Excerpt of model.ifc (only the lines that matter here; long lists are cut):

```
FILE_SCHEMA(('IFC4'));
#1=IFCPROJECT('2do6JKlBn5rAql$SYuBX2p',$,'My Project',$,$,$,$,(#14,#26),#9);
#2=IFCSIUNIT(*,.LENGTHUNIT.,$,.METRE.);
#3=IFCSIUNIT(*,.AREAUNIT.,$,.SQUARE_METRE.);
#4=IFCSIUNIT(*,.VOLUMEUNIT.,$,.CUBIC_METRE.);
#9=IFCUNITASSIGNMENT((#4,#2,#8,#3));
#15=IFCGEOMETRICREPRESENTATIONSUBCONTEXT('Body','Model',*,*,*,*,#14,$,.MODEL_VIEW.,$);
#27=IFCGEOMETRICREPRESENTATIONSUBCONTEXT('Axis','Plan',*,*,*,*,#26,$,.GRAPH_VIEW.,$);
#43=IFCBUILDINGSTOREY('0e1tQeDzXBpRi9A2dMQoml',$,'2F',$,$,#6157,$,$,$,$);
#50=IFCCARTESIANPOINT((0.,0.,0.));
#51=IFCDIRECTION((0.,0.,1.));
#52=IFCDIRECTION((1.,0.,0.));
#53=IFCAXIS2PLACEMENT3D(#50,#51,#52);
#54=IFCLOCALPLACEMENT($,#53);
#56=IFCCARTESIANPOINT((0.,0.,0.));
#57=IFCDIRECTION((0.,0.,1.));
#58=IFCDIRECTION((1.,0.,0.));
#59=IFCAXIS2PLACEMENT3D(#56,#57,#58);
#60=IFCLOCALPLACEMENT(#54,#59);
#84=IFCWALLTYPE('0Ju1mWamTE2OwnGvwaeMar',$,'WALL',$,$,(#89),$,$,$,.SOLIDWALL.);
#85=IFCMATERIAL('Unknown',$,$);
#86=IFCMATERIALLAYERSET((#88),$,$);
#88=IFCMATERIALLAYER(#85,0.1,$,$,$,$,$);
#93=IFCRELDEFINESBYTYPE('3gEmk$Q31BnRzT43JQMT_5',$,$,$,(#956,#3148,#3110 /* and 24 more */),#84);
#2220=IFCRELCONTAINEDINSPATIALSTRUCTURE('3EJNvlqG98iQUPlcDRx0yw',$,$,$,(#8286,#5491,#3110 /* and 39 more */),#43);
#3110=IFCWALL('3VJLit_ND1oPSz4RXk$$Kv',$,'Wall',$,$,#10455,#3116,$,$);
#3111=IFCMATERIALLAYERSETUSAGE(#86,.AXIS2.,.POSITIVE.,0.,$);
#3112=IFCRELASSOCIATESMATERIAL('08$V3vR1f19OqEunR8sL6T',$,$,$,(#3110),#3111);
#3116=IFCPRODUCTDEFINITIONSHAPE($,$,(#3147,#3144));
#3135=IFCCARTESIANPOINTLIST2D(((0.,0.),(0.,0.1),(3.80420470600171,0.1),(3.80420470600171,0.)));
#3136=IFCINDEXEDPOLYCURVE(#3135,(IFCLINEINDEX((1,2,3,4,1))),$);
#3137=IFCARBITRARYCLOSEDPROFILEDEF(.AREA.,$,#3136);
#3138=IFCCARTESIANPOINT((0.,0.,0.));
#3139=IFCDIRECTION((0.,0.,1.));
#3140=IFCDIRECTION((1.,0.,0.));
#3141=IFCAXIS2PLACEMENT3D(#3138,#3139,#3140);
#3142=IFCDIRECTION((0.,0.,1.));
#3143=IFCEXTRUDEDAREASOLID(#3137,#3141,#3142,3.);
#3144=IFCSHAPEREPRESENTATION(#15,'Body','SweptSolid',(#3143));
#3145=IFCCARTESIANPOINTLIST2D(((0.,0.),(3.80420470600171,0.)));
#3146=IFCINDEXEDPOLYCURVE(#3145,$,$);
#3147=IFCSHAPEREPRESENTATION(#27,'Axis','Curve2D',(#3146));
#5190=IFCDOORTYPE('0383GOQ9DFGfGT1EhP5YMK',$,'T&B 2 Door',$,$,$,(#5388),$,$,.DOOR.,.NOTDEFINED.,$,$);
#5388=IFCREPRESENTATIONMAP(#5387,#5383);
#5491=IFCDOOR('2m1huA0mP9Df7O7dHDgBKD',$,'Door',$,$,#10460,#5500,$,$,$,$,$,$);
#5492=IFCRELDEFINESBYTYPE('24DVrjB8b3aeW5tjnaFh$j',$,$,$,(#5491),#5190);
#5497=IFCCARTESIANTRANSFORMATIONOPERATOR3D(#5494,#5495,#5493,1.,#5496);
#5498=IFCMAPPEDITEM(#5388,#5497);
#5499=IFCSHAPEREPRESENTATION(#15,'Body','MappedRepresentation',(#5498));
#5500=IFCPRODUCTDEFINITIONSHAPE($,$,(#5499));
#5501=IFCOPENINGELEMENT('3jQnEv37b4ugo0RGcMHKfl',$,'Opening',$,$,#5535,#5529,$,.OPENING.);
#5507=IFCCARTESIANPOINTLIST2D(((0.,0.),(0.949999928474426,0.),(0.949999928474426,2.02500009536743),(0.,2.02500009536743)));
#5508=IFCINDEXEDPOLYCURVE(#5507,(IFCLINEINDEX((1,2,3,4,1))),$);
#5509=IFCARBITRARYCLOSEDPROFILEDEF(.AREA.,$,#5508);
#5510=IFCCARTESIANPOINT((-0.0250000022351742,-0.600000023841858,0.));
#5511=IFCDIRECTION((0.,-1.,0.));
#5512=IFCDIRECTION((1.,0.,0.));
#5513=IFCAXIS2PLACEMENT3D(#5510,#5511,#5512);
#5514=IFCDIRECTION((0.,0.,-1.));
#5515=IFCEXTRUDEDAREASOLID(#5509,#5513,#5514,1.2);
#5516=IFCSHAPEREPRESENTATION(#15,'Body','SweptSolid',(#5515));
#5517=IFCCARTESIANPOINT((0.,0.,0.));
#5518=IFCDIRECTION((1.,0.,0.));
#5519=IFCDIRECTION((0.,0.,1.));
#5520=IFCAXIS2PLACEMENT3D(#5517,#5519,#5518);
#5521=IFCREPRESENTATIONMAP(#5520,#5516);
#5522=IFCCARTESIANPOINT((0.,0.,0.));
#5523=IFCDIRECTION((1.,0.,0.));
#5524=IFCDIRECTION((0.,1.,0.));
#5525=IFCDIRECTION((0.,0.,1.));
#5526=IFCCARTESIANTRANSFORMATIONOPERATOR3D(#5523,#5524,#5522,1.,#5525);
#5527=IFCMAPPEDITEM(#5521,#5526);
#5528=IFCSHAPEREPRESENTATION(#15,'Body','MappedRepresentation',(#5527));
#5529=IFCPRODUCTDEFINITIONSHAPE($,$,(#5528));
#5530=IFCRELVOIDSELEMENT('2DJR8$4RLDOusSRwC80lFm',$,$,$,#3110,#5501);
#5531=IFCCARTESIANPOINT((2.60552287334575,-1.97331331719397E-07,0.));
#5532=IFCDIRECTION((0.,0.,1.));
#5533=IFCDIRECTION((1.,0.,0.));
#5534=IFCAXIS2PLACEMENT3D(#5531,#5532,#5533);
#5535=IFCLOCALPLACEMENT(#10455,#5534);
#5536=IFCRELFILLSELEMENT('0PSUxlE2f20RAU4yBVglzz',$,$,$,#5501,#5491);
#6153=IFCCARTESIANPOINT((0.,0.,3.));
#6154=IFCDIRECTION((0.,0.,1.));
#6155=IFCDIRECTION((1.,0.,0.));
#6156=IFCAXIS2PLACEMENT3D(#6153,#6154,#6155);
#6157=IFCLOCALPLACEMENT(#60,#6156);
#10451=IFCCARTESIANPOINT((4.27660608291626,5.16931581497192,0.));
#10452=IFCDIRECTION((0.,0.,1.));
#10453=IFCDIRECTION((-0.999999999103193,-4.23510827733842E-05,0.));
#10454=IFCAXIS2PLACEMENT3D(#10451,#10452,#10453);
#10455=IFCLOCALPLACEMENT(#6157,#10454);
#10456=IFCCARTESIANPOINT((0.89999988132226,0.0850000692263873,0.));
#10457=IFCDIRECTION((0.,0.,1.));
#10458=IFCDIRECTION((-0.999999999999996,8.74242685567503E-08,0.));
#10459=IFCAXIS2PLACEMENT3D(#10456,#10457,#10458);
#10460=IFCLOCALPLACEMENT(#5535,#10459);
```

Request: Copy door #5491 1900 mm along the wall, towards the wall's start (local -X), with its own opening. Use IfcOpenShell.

```python
import ifcopenshell
import ifcopenshell.api.feature
import ifcopenshell.api.geometry
import ifcopenshell.api.root
import ifcopenshell.geom
import ifcopenshell.util.element
import ifcopenshell.util.placement
import ifcopenshell.util.shape
import ifcopenshell.util.unit

model = ifcopenshell.open("model.ifc")
unit_scale = ifcopenshell.util.unit.calculate_unit_scale(model)
settings = ifcopenshell.geom.settings()


def volume(element):
    """Net volume in cubic metres, openings subtracted."""
    shape = ifcopenshell.geom.create_shape(settings, element)
    return ifcopenshell.util.shape.get_volume(shape.geometry)


door = model.by_guid("2m1huA0mP9Df7O7dHDgBKD")
opening = door.FillsVoids[0].RelatingOpeningElement
wall = opening.VoidsElements[0].RelatingBuildingElement
before = volume(wall)
shift = ifcopenshell.util.placement.get_local_placement(wall.ObjectPlacement)[:3, 0] * -1.9 / unit_scale

# copy_class copies the void relationship, type, container and properties, but no geometry.
new_opening = ifcopenshell.api.root.copy_class(model, product=opening)
new_opening.Representation = ifcopenshell.util.element.copy_deep(
    model, opening.Representation, exclude=["IfcGeometricRepresentationContext", "IfcRepresentationMap"]
)
new_door = ifcopenshell.api.root.copy_class(model, product=door)
new_door.Representation = ifcopenshell.util.element.copy_deep(
    model, door.Representation, exclude=["IfcGeometricRepresentationContext", "IfcRepresentationMap"]
)
ifcopenshell.api.feature.add_filling(model, opening=new_opening, element=new_door)

for old, new in ((opening, new_opening), (door, new_door)):
    matrix = ifcopenshell.util.placement.get_local_placement(old.ObjectPlacement)
    matrix[:3, 3] += shift
    ifcopenshell.api.geometry.edit_object_placement(model, product=new, matrix=matrix, is_si=False)

after = volume(wall)

print(f"wall volume {before:.3f} -> {after:.3f} m3")

model.write("model_rev.ifc")
```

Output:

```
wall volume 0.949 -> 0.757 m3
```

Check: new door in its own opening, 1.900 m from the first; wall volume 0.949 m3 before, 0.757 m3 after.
